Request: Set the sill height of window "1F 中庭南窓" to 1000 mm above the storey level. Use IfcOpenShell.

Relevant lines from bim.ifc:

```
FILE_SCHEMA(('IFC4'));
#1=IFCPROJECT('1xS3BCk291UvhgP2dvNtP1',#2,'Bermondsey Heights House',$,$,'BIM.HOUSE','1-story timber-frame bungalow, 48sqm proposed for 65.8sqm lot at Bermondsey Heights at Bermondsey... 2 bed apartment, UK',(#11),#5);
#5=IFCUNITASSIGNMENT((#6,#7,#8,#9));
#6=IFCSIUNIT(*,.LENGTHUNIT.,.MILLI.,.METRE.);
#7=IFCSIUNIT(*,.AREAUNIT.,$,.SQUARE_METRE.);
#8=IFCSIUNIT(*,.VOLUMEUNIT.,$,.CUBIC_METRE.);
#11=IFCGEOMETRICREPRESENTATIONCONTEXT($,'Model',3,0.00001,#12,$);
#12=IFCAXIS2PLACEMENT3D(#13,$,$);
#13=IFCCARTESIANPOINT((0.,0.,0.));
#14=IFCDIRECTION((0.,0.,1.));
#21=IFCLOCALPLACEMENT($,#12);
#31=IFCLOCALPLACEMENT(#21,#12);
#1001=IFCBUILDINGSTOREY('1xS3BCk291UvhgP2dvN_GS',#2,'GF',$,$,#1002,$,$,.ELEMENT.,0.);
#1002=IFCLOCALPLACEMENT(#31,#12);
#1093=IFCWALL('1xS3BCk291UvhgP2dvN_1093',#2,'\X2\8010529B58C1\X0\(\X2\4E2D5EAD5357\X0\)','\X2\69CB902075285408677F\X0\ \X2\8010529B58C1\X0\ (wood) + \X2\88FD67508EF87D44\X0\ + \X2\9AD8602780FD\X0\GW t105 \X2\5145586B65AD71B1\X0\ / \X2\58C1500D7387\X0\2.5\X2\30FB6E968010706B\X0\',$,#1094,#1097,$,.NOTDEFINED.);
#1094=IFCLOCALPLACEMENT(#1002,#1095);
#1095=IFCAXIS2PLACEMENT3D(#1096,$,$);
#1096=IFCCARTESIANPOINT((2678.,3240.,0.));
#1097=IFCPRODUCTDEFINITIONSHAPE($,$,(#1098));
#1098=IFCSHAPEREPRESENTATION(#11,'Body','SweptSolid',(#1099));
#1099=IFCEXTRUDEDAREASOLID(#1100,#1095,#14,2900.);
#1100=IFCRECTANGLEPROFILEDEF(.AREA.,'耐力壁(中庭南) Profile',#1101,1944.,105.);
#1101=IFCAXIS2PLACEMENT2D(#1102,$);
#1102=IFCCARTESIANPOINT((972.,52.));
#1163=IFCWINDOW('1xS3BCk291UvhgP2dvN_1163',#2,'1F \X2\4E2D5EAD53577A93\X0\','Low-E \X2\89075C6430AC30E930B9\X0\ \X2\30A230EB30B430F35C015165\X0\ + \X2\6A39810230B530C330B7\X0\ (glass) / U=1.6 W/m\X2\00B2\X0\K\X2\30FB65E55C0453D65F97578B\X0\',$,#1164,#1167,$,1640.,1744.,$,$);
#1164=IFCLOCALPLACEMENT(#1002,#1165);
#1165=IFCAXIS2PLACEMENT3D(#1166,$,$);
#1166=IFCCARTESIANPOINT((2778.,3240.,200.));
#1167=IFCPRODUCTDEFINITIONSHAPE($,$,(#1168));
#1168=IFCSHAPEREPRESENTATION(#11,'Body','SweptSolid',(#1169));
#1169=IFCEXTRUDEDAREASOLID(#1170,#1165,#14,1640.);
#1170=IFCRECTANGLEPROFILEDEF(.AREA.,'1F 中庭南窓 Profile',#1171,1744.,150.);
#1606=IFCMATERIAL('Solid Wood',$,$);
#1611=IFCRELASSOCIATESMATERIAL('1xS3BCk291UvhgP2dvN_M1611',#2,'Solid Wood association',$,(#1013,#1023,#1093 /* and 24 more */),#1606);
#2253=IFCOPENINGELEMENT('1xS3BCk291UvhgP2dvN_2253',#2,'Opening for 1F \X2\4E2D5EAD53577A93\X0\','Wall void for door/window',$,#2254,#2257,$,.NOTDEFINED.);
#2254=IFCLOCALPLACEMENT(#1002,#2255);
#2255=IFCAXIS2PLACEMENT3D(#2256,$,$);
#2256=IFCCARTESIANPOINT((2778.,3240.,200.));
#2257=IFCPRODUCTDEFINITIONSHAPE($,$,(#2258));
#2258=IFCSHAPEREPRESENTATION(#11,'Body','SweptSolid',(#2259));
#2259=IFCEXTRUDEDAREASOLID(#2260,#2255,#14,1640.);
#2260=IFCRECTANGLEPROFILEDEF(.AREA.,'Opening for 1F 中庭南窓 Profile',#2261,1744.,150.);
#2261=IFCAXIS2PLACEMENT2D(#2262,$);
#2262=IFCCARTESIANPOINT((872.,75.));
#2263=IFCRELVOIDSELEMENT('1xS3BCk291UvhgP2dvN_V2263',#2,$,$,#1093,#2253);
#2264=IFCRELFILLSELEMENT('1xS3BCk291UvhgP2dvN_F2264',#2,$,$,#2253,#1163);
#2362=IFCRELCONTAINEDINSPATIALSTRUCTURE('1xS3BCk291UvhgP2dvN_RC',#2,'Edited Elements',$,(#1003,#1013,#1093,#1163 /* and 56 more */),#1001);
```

```python
import numpy as np
import ifcopenshell
import ifcopenshell.api.geometry
import ifcopenshell.geom
import ifcopenshell.util.element
import ifcopenshell.util.placement
import ifcopenshell.util.shape
import ifcopenshell.util.unit

model = ifcopenshell.open("bim.ifc")
unit_scale = ifcopenshell.util.unit.calculate_unit_scale(model)

window = model.by_id(1163)
opening = window.FillsVoids[0].RelatingOpeningElement
storey = ifcopenshell.util.element.get_container(window, ifc_class="IfcBuildingStorey")
level = ifcopenshell.util.placement.get_local_placement(storey.ObjectPlacement)[2, 3]

# The opening's origin need not be at the sill, so measure its lowest point.
shape = ifcopenshell.geom.create_shape(ifcopenshell.geom.settings(), opening)
bottom = ifcopenshell.util.shape.get_shape_bottom_elevation(shape, shape.geometry) / unit_scale
dz = level + 1000.0 - bottom

shift = np.array([0.0, 0.0, dz])
# The window is not placed relative to its opening, so move both.
for product in (opening, window):
    matrix = ifcopenshell.util.placement.get_local_placement(product.ObjectPlacement)
    matrix[:3, 3] += shift
    ifcopenshell.api.geometry.edit_object_placement(model, product=product, matrix=matrix, is_si=False)

print(f"moved by {dz * unit_scale:+.3f} m")

model.write("bim_edited.ifc")
```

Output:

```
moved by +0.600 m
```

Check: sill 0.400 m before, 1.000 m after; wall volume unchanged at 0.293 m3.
